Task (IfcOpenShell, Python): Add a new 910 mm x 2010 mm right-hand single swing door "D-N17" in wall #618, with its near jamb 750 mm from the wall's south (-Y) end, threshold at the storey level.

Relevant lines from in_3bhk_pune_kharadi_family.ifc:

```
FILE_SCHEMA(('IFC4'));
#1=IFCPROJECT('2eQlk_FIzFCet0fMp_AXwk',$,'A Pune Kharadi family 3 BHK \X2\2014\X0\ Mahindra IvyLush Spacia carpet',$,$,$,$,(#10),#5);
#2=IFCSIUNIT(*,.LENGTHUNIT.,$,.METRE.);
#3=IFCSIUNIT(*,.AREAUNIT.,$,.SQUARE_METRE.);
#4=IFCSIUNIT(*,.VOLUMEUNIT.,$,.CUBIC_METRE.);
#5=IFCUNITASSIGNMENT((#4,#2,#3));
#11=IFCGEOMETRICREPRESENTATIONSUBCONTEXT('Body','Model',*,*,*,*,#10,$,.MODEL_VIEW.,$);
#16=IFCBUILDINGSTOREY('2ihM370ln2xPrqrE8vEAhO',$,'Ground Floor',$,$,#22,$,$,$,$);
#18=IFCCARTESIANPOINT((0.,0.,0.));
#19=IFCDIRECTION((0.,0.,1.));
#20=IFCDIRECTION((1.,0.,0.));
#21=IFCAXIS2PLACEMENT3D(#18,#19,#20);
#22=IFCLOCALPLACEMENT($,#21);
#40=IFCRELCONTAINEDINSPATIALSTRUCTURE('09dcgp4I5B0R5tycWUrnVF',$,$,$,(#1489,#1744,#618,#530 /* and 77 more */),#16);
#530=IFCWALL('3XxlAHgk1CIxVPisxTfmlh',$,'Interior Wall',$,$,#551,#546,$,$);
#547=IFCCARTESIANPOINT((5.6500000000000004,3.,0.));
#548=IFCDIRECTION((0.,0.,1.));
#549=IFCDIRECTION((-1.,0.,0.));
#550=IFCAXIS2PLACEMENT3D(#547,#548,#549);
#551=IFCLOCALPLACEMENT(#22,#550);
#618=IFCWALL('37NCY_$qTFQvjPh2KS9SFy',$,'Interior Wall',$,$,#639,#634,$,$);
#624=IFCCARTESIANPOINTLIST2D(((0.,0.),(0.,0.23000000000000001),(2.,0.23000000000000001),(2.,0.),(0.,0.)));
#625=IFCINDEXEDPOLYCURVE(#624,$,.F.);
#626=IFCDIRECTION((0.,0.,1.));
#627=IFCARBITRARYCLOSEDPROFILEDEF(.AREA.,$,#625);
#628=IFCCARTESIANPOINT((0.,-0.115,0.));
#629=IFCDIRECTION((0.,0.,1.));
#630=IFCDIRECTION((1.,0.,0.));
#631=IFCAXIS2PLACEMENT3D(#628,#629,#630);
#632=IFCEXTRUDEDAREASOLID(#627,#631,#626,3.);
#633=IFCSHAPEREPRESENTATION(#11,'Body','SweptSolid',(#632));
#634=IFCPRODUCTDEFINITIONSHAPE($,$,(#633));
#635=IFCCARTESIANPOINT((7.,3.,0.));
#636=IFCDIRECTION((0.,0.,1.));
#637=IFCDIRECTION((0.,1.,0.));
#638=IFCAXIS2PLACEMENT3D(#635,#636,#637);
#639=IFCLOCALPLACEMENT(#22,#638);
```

```python
import numpy as np
import ifcopenshell
import ifcopenshell.api.feature
import ifcopenshell.api.geometry
import ifcopenshell.api.root
import ifcopenshell.api.spatial
import ifcopenshell.geom
import ifcopenshell.util.element
import ifcopenshell.util.placement
import ifcopenshell.util.representation
import ifcopenshell.util.shape
import ifcopenshell.util.unit

model = ifcopenshell.open("in_3bhk_pune_kharadi_family.ifc")
unit_scale = ifcopenshell.util.unit.calculate_unit_scale(model)
settings = ifcopenshell.geom.settings()


def volume(element):
    """Net volume in cubic metres, openings subtracted."""
    shape = ifcopenshell.geom.create_shape(settings, element)
    return ifcopenshell.util.shape.get_volume(shape.geometry)


wall = model.by_guid("37NCY_$qTFQvjPh2KS9SFy")
storey = ifcopenshell.util.element.get_container(wall, ifc_class="IfcBuildingStorey")
context = ifcopenshell.util.representation.get_context(model, "Model", "Body", "MODEL_VIEW")
before = volume(wall)

width, height, from_end, sill = 0.91, 2.01, 0.75, 0.0  # metres

# The wall runs along its own X axis, and the end named is its -X end.
wall_shape = ifcopenshell.geom.create_shape(settings, wall)
x, y, z = ifcopenshell.util.shape.get_vertices(wall_shape.geometry).T
start = x.min() + from_end
face, thickness = float(y.min()), float(y.max() - y.min())
wall_matrix = ifcopenshell.util.placement.get_local_placement(wall.ObjectPlacement)
level = ifcopenshell.util.placement.get_local_placement(storey.ObjectPlacement)[2, 3]


def in_wall(x, y):
    """Placement at x, y metres in the wall's axes, at sill height."""
    matrix = wall_matrix.copy()
    matrix[:, 3] = wall_matrix @ np.array([x / unit_scale, y / unit_scale, 0.0, 1.0])
    matrix[2, 3] = level + sill / unit_scale
    return matrix


# Opening: a box that overshoots both wall faces by 50 mm.
opening = ifcopenshell.api.root.create_entity(model, ifc_class="IfcOpeningElement", predefined_type="OPENING")
box = ifcopenshell.api.geometry.add_wall_representation(
    model, context=context, length=width, height=height, thickness=thickness + 0.1
)
ifcopenshell.api.geometry.assign_representation(model, product=opening, representation=box)
ifcopenshell.api.geometry.edit_object_placement(model, product=opening, matrix=in_wall(start, face - 0.05), is_si=False)
ifcopenshell.api.feature.add_feature(model, feature=opening, element=wall)

door = ifcopenshell.api.root.create_entity(model, ifc_class="IfcDoor", name="D-N17", predefined_type="DOOR")
door.OverallWidth, door.OverallHeight = width / unit_scale, height / unit_scale
door.OperationType = "SINGLE_SWING_RIGHT"
body = ifcopenshell.api.geometry.add_door_representation(
    model,
    context=context,
    overall_width=door.OverallWidth,
    overall_height=door.OverallHeight,
    operation_type="SINGLE_SWING_RIGHT",
    lining_properties={"LiningDepth": thickness / unit_scale, "ThresholdDepth": thickness / unit_scale},
)
ifcopenshell.api.geometry.assign_representation(model, product=door, representation=body)
ifcopenshell.api.spatial.assign_container(model, products=[door], relating_structure=storey)
ifcopenshell.api.feature.add_filling(model, opening=opening, element=door)

# The lining spans the wall, so the door starts at the wall face.
ifcopenshell.api.geometry.edit_object_placement(model, product=door, matrix=in_wall(start, face), is_si=False)

after = volume(wall)

print(f"wall volume {before:.3f} -> {after:.3f} m3")

model.write("in_3bhk_pune_kharadi_family-out.ifc")
```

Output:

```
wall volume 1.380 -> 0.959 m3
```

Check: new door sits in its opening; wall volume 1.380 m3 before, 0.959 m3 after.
